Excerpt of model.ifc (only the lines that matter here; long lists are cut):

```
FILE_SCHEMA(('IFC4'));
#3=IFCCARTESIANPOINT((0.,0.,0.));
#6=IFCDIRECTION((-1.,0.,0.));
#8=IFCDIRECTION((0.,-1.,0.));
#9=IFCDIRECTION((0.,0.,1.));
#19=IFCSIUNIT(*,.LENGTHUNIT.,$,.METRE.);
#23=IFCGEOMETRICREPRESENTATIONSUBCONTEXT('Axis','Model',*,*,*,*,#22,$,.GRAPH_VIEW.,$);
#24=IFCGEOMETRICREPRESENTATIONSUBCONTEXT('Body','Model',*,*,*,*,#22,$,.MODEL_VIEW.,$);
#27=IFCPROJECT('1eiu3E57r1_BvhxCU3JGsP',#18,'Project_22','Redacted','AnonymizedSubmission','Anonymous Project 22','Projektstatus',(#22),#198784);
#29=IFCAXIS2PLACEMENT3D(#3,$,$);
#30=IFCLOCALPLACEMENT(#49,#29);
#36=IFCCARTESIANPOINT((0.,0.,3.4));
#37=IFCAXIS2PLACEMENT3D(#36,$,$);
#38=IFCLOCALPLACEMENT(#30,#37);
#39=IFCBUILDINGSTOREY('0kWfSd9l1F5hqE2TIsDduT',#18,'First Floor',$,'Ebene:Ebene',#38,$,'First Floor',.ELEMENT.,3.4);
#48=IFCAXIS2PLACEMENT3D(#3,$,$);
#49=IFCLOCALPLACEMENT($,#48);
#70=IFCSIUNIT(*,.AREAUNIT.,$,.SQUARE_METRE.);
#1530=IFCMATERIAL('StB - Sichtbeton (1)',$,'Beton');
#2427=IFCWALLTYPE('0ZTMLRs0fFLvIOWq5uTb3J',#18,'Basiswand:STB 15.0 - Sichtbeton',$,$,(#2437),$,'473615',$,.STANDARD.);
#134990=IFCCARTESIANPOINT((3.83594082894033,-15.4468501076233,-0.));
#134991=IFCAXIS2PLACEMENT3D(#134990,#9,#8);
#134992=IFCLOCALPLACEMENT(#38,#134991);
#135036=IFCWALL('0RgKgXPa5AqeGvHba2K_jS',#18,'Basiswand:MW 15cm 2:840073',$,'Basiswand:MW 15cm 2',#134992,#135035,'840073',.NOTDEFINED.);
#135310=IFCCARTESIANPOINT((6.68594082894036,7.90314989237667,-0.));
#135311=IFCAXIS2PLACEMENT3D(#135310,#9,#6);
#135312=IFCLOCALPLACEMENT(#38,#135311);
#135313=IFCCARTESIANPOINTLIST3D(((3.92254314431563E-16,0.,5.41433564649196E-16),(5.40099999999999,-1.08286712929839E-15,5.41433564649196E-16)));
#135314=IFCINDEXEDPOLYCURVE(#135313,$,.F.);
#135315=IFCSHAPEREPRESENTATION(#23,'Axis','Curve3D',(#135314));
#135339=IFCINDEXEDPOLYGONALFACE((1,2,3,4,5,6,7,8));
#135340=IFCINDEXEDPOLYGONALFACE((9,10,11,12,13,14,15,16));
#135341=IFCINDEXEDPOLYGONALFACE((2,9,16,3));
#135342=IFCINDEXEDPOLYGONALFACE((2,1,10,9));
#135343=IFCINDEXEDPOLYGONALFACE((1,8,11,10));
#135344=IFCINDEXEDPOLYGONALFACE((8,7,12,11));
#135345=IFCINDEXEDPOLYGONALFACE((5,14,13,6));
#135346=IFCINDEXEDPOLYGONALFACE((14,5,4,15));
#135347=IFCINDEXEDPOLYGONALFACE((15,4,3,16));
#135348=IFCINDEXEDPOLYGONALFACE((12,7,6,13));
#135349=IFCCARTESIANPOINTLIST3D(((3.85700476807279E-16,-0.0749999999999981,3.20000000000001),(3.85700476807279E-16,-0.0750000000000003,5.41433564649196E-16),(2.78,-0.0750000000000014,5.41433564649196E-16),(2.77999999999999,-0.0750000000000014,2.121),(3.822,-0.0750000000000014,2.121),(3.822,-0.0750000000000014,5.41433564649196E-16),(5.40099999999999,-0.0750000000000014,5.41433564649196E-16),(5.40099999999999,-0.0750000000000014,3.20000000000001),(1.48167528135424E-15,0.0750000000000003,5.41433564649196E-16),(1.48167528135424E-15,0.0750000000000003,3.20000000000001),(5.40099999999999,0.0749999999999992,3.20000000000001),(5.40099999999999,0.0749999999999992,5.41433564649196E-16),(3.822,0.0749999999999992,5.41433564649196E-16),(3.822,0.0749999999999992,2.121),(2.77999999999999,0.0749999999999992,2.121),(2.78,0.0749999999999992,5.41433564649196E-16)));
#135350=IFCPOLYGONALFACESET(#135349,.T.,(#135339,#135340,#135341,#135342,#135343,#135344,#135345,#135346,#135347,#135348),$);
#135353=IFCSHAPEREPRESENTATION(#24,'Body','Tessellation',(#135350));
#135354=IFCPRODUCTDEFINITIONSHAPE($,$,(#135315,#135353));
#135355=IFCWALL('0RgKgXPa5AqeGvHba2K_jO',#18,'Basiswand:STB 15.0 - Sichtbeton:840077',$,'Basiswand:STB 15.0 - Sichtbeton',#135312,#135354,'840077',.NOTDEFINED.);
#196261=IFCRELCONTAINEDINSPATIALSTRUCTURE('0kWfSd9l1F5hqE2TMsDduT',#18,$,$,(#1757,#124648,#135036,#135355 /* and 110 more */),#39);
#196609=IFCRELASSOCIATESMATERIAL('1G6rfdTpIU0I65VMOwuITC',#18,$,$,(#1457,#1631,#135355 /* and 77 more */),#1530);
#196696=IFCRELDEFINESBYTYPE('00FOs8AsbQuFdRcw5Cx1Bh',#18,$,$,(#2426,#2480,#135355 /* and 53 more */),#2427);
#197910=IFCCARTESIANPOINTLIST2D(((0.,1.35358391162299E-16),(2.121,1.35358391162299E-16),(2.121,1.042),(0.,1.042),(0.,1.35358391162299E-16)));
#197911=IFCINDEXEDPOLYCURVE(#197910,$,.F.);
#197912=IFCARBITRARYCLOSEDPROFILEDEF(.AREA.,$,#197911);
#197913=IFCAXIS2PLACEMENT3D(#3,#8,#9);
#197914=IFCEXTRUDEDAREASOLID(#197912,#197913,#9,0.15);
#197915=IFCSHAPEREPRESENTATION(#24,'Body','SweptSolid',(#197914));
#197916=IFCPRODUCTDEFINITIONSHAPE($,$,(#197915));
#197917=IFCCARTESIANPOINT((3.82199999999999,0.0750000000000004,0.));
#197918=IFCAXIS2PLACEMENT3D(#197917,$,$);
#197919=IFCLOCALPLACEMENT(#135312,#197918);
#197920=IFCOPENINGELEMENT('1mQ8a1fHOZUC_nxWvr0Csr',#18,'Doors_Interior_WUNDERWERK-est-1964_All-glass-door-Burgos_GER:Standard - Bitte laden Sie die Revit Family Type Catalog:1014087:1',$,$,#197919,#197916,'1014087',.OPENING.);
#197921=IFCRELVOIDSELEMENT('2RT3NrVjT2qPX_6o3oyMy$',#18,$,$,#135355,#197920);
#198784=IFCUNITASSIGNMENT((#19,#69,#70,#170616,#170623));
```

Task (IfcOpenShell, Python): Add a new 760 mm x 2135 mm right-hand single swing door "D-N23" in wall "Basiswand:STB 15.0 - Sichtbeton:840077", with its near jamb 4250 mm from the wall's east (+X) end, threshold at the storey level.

```python
import numpy as np
import ifcopenshell
import ifcopenshell.api.feature
import ifcopenshell.api.geometry
import ifcopenshell.api.root
import ifcopenshell.api.spatial
import ifcopenshell.geom
import ifcopenshell.util.element
import ifcopenshell.util.placement
import ifcopenshell.util.representation
import ifcopenshell.util.shape
import ifcopenshell.util.unit

model = ifcopenshell.open("model.ifc")
unit_scale = ifcopenshell.util.unit.calculate_unit_scale(model)
settings = ifcopenshell.geom.settings()


def volume(element):
    """Net volume in cubic metres, openings subtracted."""
    shape = ifcopenshell.geom.create_shape(settings, element)
    return ifcopenshell.util.shape.get_volume(shape.geometry)


wall = model.by_guid("0RgKgXPa5AqeGvHba2K_jO")
storey = ifcopenshell.util.element.get_container(wall, ifc_class="IfcBuildingStorey")
context = ifcopenshell.util.representation.get_context(model, "Model", "Body", "MODEL_VIEW")
before = volume(wall)

width, height, from_end, sill = 0.76, 2.135, 4.25, 0.0  # metres

# The wall runs along its own X axis, and the end named is its -X end.
wall_shape = ifcopenshell.geom.create_shape(settings, wall)
x, y, z = ifcopenshell.util.shape.get_vertices(wall_shape.geometry).T
start = x.min() + from_end
face, thickness = float(y.min()), float(y.max() - y.min())
wall_matrix = ifcopenshell.util.placement.get_local_placement(wall.ObjectPlacement)
level = ifcopenshell.util.placement.get_local_placement(storey.ObjectPlacement)[2, 3]


def in_wall(x, y):
    """Placement at x, y metres in the wall's axes, at sill height."""
    matrix = wall_matrix.copy()
    matrix[:, 3] = wall_matrix @ np.array([x / unit_scale, y / unit_scale, 0.0, 1.0])
    matrix[2, 3] = level + sill / unit_scale
    return matrix


# Opening: a box that overshoots both wall faces by 50 mm.
opening = ifcopenshell.api.root.create_entity(model, ifc_class="IfcOpeningElement", predefined_type="OPENING")
box = ifcopenshell.api.geometry.add_wall_representation(
    model, context=context, length=width, height=height, thickness=thickness + 0.1
)
ifcopenshell.api.geometry.assign_representation(model, product=opening, representation=box)
ifcopenshell.api.geometry.edit_object_placement(model, product=opening, matrix=in_wall(start, face - 0.05), is_si=False)
ifcopenshell.api.feature.add_feature(model, feature=opening, element=wall)

door = ifcopenshell.api.root.create_entity(model, ifc_class="IfcDoor", name="D-N23", predefined_type="DOOR")
door.OverallWidth, door.OverallHeight = width / unit_scale, height / unit_scale
door.OperationType = "SINGLE_SWING_RIGHT"
body = ifcopenshell.api.geometry.add_door_representation(
    model,
    context=context,
    overall_width=door.OverallWidth,
    overall_height=door.OverallHeight,
    operation_type="SINGLE_SWING_RIGHT",
    lining_properties={"LiningDepth": thickness / unit_scale, "ThresholdDepth": thickness / unit_scale},
)
ifcopenshell.api.geometry.assign_representation(model, product=door, representation=body)
ifcopenshell.api.spatial.assign_container(model, products=[door], relating_structure=storey)
ifcopenshell.api.feature.add_filling(model, opening=opening, element=door)

# The lining spans the wall, so the door starts at the wall face.
ifcopenshell.api.geometry.edit_object_placement(model, product=door, matrix=in_wall(start, face), is_si=False)

after = volume(wall)

print(f"wall volume {before:.3f} -> {after:.3f} m3")

model.write("model_rev.ifc")
```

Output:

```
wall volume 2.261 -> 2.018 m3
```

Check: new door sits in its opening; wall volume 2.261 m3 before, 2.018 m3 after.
